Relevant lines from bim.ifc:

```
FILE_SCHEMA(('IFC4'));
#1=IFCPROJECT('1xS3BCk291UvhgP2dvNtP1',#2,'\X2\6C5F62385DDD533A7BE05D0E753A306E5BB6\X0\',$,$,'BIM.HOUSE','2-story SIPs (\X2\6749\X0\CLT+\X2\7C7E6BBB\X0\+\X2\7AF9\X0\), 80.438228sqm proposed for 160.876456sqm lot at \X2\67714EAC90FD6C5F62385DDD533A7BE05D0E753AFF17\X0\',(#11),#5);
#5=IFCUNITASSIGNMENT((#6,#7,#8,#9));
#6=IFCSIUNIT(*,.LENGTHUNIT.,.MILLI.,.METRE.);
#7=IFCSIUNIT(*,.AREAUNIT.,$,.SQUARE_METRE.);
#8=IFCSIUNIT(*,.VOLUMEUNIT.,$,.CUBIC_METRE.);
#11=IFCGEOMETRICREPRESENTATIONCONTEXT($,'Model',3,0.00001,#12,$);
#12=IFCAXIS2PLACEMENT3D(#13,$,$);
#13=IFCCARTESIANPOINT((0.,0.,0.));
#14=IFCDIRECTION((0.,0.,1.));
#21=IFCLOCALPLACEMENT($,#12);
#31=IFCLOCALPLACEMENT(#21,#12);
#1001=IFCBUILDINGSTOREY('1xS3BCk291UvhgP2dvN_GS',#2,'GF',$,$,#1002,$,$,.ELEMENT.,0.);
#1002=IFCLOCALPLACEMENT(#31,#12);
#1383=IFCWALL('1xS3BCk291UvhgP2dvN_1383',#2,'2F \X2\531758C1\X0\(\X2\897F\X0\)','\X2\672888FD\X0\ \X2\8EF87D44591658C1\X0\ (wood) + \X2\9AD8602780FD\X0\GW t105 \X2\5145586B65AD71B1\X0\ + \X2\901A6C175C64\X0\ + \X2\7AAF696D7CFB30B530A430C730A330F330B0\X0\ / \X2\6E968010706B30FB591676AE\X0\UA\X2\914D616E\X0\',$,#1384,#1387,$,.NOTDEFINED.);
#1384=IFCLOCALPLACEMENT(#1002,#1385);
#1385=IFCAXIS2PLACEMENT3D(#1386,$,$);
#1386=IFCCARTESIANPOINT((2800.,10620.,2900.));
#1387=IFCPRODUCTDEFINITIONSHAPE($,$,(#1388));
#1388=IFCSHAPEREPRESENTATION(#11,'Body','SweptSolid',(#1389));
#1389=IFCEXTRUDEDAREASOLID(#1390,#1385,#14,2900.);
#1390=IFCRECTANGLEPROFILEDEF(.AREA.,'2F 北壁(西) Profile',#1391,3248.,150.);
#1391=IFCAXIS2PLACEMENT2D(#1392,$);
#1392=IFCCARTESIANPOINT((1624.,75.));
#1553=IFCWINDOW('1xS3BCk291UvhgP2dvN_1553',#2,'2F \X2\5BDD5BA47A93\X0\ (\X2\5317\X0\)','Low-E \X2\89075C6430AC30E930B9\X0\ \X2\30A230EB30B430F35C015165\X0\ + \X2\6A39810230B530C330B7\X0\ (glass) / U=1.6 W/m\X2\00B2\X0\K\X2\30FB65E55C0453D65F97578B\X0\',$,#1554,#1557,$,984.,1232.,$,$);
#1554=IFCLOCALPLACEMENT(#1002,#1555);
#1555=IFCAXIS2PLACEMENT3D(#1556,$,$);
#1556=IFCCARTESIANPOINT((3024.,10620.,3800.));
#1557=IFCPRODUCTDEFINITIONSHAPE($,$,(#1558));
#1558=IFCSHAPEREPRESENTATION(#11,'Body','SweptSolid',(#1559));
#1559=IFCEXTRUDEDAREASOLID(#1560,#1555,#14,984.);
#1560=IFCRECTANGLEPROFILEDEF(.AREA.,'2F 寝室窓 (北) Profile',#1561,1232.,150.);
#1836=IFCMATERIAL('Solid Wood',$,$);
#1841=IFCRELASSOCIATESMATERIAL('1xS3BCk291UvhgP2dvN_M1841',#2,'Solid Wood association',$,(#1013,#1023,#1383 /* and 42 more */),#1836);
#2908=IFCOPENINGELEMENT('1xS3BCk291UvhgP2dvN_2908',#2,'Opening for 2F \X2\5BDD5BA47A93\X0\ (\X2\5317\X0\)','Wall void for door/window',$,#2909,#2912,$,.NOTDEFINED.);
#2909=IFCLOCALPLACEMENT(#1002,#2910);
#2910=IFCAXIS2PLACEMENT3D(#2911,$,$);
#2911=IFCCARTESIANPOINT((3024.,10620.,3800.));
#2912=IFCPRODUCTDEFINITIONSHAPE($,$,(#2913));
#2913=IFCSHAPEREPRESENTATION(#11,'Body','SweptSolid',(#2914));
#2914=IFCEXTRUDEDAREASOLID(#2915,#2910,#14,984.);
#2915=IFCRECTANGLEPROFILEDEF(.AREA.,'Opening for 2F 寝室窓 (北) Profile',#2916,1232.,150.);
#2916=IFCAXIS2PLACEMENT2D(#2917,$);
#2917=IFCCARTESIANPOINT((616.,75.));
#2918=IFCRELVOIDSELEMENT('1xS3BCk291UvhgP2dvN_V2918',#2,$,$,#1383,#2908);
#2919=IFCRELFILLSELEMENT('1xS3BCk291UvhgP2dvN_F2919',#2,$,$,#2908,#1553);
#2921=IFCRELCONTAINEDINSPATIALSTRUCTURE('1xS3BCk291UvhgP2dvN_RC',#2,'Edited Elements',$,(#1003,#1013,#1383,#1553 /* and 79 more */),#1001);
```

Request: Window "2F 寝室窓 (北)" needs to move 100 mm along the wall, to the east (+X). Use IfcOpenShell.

```python
import ifcopenshell
import ifcopenshell.api.geometry
import ifcopenshell.util.placement
import ifcopenshell.util.unit

model = ifcopenshell.open("bim.ifc")
unit_scale = ifcopenshell.util.unit.calculate_unit_scale(model)

window = model.by_guid("1xS3BCk291UvhgP2dvN_1553")
opening = window.FillsVoids[0].RelatingOpeningElement
wall = opening.VoidsElements[0].RelatingBuildingElement

wall_matrix = ifcopenshell.util.placement.get_local_placement(wall.ObjectPlacement)
shift = wall_matrix[:3, 0] * 0.1 / unit_scale
before = ifcopenshell.util.placement.get_local_placement(window.ObjectPlacement)[:3, 3].copy()

# The window is not placed relative to its opening, so move both.
for product in (opening, window):
    matrix = ifcopenshell.util.placement.get_local_placement(product.ObjectPlacement)
    matrix[:3, 3] += shift
    ifcopenshell.api.geometry.edit_object_placement(model, product=product, matrix=matrix, is_si=False)

after = ifcopenshell.util.placement.get_local_placement(window.ObjectPlacement)[:3, 3]
print("window moved by", (after - before).round(3) + 0.0)

model.write("bim-out.ifc")
```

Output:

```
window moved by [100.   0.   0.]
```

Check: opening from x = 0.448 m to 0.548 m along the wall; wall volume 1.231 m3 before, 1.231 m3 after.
